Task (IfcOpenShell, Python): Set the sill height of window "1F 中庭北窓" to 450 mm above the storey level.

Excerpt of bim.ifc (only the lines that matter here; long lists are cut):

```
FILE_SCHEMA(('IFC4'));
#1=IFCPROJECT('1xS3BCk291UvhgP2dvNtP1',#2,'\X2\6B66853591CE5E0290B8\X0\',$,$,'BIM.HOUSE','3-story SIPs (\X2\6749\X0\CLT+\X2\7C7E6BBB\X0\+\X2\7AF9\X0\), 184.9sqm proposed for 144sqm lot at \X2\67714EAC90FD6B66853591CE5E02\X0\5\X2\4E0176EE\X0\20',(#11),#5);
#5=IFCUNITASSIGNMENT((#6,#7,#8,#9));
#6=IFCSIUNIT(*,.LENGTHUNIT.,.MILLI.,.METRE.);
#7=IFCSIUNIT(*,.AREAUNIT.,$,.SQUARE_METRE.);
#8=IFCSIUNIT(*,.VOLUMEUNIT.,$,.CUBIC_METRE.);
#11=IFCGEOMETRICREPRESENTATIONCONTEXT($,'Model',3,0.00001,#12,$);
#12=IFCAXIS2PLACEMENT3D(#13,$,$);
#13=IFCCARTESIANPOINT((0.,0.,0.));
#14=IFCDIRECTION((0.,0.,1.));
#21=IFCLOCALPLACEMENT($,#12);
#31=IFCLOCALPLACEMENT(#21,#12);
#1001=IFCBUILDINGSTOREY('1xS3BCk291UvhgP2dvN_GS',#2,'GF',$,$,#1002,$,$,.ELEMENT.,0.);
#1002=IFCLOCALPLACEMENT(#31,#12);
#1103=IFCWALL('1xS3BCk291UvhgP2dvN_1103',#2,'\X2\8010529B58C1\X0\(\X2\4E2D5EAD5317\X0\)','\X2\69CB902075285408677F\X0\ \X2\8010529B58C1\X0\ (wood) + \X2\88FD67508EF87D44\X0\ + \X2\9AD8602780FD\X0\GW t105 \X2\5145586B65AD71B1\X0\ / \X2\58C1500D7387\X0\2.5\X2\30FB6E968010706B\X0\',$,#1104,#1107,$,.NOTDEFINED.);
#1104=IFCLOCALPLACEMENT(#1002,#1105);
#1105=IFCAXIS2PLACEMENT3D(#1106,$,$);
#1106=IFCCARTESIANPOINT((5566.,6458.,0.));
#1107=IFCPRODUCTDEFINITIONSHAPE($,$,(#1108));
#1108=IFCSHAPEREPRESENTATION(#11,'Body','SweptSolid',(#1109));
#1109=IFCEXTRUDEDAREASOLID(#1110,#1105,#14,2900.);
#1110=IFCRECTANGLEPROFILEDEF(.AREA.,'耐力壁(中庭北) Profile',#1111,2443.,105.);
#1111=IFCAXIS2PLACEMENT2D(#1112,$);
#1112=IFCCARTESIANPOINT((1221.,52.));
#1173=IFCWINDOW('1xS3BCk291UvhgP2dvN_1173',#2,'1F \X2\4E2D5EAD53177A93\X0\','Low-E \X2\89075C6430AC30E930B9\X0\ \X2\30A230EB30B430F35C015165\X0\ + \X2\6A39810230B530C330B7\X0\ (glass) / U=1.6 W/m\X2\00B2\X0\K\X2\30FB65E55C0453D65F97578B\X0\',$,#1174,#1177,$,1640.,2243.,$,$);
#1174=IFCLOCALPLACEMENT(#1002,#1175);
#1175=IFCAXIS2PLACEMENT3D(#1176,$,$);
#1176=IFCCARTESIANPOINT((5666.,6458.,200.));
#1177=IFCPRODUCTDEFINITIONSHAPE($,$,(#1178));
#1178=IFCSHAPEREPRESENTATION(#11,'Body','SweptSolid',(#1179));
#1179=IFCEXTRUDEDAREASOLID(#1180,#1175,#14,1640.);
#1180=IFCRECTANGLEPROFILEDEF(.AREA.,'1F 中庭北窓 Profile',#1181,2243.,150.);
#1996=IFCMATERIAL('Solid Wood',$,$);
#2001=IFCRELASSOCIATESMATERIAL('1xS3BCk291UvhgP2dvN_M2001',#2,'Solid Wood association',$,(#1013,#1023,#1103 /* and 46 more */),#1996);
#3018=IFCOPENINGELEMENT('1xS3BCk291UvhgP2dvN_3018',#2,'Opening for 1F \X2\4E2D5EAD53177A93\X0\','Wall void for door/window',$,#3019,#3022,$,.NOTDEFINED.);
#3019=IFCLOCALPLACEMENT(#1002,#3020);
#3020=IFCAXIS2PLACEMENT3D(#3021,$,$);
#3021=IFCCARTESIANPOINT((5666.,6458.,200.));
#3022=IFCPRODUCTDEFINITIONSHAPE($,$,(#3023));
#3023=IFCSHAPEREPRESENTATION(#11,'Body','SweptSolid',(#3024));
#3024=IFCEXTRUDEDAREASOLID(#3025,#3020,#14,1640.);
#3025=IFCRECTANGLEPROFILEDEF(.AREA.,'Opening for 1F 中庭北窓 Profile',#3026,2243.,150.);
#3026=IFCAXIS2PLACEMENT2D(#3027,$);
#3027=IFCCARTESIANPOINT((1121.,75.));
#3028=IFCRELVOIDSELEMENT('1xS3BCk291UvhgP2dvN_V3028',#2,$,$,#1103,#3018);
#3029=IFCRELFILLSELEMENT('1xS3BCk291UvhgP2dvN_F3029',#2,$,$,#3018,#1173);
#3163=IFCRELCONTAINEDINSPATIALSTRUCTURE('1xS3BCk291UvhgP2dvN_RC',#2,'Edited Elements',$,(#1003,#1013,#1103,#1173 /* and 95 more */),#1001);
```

```python
import numpy as np
import ifcopenshell
import ifcopenshell.api.geometry
import ifcopenshell.geom
import ifcopenshell.util.element
import ifcopenshell.util.placement
import ifcopenshell.util.shape
import ifcopenshell.util.unit

model = ifcopenshell.open("bim.ifc")
unit_scale = ifcopenshell.util.unit.calculate_unit_scale(model)

window = model.by_id(1173)
opening = window.FillsVoids[0].RelatingOpeningElement
storey = ifcopenshell.util.element.get_container(window, ifc_class="IfcBuildingStorey")
level = ifcopenshell.util.placement.get_local_placement(storey.ObjectPlacement)[2, 3]

# The opening's origin need not be at the sill, so measure its lowest point.
shape = ifcopenshell.geom.create_shape(ifcopenshell.geom.settings(), opening)
bottom = ifcopenshell.util.shape.get_shape_bottom_elevation(shape, shape.geometry) / unit_scale
dz = level + 450.0 - bottom

shift = np.array([0.0, 0.0, dz])
# The window is not placed relative to its opening, so move both.
for product in (opening, window):
    matrix = ifcopenshell.util.placement.get_local_placement(product.ObjectPlacement)
    matrix[:3, 3] += shift
    ifcopenshell.api.geometry.edit_object_placement(model, product=product, matrix=matrix, is_si=False)

print(f"moved by {dz * unit_scale:+.3f} m")

model.write("bim_rev.ifc")
```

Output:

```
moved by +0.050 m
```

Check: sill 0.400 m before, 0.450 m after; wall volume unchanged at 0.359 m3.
